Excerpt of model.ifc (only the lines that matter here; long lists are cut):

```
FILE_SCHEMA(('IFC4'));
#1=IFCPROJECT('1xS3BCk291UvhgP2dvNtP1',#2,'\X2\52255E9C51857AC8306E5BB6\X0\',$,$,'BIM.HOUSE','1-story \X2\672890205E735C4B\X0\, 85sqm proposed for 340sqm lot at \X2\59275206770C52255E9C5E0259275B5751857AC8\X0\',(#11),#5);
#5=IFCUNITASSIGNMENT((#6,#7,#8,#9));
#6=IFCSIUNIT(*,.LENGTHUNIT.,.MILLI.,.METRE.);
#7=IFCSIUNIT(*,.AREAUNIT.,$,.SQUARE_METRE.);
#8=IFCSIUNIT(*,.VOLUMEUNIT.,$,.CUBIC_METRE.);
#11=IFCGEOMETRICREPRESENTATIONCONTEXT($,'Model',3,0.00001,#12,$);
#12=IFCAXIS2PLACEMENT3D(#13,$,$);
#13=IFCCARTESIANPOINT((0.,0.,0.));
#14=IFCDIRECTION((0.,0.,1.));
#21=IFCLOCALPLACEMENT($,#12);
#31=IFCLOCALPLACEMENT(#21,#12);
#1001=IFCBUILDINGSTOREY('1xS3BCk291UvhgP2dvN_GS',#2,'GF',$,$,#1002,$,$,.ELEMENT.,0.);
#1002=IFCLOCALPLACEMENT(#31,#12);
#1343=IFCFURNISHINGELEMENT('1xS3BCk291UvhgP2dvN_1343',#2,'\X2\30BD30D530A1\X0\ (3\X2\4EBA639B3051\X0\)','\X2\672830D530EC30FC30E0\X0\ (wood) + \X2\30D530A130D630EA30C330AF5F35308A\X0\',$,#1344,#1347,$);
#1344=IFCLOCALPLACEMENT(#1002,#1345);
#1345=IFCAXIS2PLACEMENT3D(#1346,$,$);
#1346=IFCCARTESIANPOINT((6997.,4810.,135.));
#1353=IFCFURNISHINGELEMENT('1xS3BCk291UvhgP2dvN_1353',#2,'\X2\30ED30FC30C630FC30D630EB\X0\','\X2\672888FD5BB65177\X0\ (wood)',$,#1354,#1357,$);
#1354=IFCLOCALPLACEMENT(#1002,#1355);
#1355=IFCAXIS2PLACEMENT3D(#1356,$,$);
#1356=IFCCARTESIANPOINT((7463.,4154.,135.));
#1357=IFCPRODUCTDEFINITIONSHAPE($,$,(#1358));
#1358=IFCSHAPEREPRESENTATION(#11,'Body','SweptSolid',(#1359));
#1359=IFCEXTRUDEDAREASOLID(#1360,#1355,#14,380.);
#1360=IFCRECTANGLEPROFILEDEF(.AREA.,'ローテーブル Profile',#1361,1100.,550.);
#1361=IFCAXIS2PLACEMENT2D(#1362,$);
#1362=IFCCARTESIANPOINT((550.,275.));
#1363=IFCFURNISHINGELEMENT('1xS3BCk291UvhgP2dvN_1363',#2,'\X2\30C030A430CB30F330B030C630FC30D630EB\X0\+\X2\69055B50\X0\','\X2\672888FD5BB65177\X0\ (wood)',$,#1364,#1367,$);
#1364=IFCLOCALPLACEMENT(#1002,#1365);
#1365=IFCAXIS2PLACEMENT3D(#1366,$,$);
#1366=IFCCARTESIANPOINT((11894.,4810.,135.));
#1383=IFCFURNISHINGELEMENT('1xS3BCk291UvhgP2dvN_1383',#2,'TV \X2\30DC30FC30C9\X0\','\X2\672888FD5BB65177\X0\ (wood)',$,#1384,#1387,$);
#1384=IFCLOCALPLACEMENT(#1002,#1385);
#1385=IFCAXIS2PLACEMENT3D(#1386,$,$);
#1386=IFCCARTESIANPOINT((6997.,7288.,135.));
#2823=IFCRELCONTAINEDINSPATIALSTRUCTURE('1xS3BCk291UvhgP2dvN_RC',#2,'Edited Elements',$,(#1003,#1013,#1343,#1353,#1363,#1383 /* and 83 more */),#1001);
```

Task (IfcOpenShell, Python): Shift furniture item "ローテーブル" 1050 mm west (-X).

```python
import ifcopenshell
import ifcopenshell.api.geometry
import ifcopenshell.util.placement

model = ifcopenshell.open("model.ifc")

item = model.by_guid("1xS3BCk291UvhgP2dvN_1353")
matrix = ifcopenshell.util.placement.get_local_placement(item.ObjectPlacement)
matrix[0, 3] -= 1050.0
ifcopenshell.api.geometry.edit_object_placement(model, product=item, matrix=matrix, is_si=False)

print(ifcopenshell.util.placement.get_local_placement(item.ObjectPlacement).round(3) + 0.0)

model.write("model-out.ifc")
```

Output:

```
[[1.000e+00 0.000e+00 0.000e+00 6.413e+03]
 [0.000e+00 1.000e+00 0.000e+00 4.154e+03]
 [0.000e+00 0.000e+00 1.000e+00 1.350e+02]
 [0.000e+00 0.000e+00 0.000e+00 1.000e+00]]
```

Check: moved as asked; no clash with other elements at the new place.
